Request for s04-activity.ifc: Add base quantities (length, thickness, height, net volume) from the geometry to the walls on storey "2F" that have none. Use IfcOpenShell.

First a look at what the model holds.

```python
import ifcopenshell
import ifcopenshell.util.element
import ifcopenshell.util.unit

model = ifcopenshell.open("s04-activity.ifc")
print(model.schema)
for unit_type in ("LENGTHUNIT", "AREAUNIT", "VOLUMEUNIT"):
    print(unit_type, ifcopenshell.util.unit.calculate_unit_scale(model, unit_type))
storey = next(s for s in model.by_type("IfcBuildingStorey") if s.Name == "2F")
walls = [e for e in ifcopenshell.util.element.get_decomposition(storey) if e.is_a("IfcWall")]
for e in sorted(walls, key=lambda e: e.id()):
    print(e.id(), e.is_a(), e.Name, list(ifcopenshell.util.element.get_psets(e, qtos_only=True)), sep=" | ")
```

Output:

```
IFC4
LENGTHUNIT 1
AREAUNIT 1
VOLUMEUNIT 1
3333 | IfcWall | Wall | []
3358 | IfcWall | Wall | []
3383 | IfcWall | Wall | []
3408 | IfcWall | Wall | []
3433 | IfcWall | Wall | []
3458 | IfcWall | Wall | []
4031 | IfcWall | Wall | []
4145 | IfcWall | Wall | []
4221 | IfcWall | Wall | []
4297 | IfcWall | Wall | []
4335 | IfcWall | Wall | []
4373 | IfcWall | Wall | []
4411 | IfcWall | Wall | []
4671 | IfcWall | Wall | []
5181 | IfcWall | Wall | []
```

```python
import ifcopenshell
import ifcopenshell.api.pset
import ifcopenshell.geom
import ifcopenshell.util.element
import ifcopenshell.util.shape
import ifcopenshell.util.unit

model = ifcopenshell.open("s04-activity.ifc")
unit_scale = ifcopenshell.util.unit.calculate_unit_scale(model)
volume_scale = ifcopenshell.util.unit.calculate_unit_scale(model, "VOLUMEUNIT")
settings = ifcopenshell.geom.settings()

storey = next(s for s in model.by_type("IfcBuildingStorey") if s.Name == "2F")
walls = [e for e in ifcopenshell.util.element.get_decomposition(storey) if e.is_a("IfcWall")]

for e in sorted(walls, key=lambda e: e.id()):
    if ifcopenshell.util.element.get_psets(e, qtos_only=True, should_inherit=False):
        continue
    # Geometry comes back in metres, in the element's own axes.
    shape = ifcopenshell.geom.create_shape(settings, e)
    values = {
        "Length": ifcopenshell.util.shape.get_x(shape.geometry) / unit_scale,
        "Width": ifcopenshell.util.shape.get_y(shape.geometry) / unit_scale,
        "Height": ifcopenshell.util.shape.get_z(shape.geometry) / unit_scale,
        "NetVolume": ifcopenshell.util.shape.get_volume(shape.geometry) / volume_scale,
    }
    qto = ifcopenshell.api.pset.add_qto(model, product=e, name="Qto_WallBaseQuantities")
    ifcopenshell.api.pset.edit_qto(model, qto=qto, properties=values)
    print(e.id(), {k: round(v, 3) for k, v in values.items()})

model.write("s04-activity_edited.ifc")
```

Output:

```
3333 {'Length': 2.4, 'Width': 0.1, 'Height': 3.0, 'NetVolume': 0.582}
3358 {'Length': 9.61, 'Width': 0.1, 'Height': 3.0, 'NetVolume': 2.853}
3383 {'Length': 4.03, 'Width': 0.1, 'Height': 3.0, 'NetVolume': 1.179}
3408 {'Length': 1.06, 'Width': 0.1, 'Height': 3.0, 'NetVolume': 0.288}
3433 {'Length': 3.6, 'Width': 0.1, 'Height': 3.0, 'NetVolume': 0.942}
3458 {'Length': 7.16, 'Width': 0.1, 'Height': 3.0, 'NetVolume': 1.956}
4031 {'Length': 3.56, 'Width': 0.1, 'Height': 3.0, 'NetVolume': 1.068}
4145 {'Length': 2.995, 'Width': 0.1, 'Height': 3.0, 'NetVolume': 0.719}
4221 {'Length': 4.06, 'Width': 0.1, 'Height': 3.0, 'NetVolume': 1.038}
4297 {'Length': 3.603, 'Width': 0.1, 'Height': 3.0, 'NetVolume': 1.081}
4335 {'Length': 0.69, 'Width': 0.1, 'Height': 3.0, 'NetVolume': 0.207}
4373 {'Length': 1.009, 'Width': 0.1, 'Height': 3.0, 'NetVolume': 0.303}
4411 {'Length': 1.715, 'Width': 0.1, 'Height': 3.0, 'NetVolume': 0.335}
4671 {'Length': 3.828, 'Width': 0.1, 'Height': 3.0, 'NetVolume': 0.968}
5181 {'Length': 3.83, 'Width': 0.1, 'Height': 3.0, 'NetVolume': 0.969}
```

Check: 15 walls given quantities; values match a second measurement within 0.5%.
